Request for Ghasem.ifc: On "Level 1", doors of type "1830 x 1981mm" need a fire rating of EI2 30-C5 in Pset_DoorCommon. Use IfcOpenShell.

First a look at what the model holds.

```python
import ifcopenshell
import ifcopenshell.util.element

model = ifcopenshell.open("Ghasem.ifc")
print(model.schema)
storey = next(s for s in model.by_type("IfcBuildingStorey") if s.Name == "Level 1")
doors = [e for e in ifcopenshell.util.element.get_decomposition(storey) if e.is_a("IfcDoor")]
seen = {}
for e in doors:
    element_type = ifcopenshell.util.element.get_type(e)
    key = (element_type.Name if element_type != e and element_type else None, ifcopenshell.util.element.get_pset(e, "Pset_DoorCommon", "FireRating"))
    seen[key] = seen.get(key, 0) + 1
for (name, value), count in sorted(seen.items(), key=str):
    print(count, "x", name, "|", value)
```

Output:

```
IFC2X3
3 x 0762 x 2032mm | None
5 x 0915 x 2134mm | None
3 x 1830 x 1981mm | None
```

```python
import ifcopenshell
import ifcopenshell.api.pset
import ifcopenshell.util.element

model = ifcopenshell.open("Ghasem.ifc")

storey = next(s for s in model.by_type("IfcBuildingStorey") if s.Name == "Level 1")
doors = [e for e in ifcopenshell.util.element.get_decomposition(storey) if e.is_a("IfcDoor")]

count = 0
for e in doors:
    element_type = ifcopenshell.util.element.get_type(e)
    if element_type in (None, e) or element_type.Name != "1830 x 1981mm":
        continue
    # add_pset returns the element's existing set when there is one.
    pset = ifcopenshell.api.pset.add_pset(model, product=e, name="Pset_DoorCommon")
    ifcopenshell.api.pset.edit_pset(model, pset=pset, properties={"FireRating": "EI2 30-C5"})
    count += 1

print(count, "doors updated")

model.write("Ghasem-out.ifc")
```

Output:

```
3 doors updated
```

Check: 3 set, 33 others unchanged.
